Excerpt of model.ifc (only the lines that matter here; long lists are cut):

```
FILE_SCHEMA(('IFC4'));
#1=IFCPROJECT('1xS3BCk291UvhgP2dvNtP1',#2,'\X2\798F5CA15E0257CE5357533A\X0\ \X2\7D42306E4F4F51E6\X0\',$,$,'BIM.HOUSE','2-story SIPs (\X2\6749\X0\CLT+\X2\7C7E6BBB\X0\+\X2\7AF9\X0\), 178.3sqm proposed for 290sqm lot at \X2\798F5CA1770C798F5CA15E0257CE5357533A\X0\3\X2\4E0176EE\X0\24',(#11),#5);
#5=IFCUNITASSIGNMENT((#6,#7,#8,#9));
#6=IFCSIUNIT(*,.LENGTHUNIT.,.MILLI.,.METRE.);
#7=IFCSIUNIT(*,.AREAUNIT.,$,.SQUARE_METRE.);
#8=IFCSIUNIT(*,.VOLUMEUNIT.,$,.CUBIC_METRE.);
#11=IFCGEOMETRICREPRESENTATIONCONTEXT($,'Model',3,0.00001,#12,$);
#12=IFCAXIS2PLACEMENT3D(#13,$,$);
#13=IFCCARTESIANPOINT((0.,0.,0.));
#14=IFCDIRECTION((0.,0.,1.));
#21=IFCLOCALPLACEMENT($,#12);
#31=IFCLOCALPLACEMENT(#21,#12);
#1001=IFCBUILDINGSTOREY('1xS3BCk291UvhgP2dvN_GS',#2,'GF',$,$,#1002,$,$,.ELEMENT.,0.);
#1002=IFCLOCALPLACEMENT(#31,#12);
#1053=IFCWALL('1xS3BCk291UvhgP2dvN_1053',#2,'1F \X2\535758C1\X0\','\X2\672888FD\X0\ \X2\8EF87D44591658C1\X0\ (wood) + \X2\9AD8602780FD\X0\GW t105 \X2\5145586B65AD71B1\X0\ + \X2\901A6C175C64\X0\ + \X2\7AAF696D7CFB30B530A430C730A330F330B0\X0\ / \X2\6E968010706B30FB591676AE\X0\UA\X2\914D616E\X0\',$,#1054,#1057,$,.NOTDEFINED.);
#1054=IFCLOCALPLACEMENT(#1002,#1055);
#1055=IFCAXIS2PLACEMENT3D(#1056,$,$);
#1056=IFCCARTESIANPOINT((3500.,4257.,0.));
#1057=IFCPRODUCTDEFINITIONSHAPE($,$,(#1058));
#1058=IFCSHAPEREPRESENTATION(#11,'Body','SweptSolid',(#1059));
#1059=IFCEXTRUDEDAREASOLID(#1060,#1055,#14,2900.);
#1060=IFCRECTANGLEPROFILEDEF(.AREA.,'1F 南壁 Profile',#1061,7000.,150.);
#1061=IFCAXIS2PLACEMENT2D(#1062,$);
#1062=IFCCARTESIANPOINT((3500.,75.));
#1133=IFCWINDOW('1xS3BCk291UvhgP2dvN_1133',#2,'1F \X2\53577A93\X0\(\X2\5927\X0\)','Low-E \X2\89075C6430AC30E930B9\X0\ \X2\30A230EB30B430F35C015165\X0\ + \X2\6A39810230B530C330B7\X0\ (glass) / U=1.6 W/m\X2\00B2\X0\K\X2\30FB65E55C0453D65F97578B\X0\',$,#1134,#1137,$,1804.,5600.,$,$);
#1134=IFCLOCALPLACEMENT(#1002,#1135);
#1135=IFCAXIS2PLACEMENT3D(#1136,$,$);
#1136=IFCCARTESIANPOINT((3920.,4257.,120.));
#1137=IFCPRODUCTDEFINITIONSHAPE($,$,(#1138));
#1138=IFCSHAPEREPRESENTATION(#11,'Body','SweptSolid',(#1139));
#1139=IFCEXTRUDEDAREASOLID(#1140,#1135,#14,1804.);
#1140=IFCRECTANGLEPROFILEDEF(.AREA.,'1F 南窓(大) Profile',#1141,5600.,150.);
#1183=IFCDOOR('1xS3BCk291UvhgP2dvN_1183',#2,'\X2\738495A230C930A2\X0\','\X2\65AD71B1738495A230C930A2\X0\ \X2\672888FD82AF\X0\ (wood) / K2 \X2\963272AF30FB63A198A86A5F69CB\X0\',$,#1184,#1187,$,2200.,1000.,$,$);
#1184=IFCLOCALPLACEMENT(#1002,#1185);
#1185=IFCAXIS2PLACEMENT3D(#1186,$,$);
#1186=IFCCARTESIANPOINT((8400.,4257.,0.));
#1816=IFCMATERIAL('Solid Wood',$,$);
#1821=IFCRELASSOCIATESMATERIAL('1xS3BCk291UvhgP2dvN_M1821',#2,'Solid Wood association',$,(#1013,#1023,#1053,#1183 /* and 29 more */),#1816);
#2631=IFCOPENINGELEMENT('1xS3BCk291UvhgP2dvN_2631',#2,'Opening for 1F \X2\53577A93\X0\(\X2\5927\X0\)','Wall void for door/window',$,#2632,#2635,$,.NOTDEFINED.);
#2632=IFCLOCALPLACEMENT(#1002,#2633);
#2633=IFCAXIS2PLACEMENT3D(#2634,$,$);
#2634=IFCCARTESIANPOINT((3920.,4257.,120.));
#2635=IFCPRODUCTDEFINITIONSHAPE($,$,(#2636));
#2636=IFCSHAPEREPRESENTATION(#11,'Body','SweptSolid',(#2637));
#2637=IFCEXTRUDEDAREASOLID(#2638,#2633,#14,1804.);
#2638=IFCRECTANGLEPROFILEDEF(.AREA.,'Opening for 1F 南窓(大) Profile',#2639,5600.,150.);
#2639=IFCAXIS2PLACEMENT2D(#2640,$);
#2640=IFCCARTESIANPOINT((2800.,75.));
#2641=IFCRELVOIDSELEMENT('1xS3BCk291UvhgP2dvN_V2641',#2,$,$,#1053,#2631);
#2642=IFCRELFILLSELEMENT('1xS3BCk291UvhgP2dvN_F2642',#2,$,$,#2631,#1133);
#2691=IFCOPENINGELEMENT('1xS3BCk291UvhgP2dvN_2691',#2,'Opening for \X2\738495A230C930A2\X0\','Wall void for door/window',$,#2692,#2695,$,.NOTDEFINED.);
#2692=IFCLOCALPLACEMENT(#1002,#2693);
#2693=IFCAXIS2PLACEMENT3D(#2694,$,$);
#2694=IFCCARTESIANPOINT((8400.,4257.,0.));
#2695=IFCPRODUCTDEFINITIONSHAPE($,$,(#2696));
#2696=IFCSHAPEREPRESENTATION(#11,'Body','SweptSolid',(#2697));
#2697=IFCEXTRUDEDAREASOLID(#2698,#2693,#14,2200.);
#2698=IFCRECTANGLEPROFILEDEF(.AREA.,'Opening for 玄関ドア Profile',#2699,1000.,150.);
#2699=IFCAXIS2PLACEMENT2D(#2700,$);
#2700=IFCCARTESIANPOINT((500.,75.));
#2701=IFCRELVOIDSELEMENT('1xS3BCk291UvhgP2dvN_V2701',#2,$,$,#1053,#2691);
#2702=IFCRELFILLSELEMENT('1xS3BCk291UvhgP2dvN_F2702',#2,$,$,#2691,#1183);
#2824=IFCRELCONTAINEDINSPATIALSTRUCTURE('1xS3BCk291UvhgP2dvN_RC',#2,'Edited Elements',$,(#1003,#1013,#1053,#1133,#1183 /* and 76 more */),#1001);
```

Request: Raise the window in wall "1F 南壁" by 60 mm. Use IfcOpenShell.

```python
import numpy as np
import ifcopenshell
import ifcopenshell.api.geometry
import ifcopenshell.util.placement
import ifcopenshell.util.unit

model = ifcopenshell.open("model.ifc")
unit_scale = ifcopenshell.util.unit.calculate_unit_scale(model)

window = model.by_id(1133)
opening = window.FillsVoids[0].RelatingOpeningElement
dz = 0.06 / unit_scale

shift = np.array([0.0, 0.0, dz])
# The window is not placed relative to its opening, so move both.
for product in (opening, window):
    matrix = ifcopenshell.util.placement.get_local_placement(product.ObjectPlacement)
    matrix[:3, 3] += shift
    ifcopenshell.api.geometry.edit_object_placement(model, product=product, matrix=matrix, is_si=False)

print(f"moved by {dz * unit_scale:+.3f} m")

model.write("model_updated.ifc")
```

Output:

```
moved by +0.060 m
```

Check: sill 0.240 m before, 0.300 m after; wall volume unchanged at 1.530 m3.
